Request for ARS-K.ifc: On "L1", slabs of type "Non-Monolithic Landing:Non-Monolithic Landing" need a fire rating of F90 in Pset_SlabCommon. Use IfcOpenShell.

First a look at what the model holds.

```python
import ifcopenshell
import ifcopenshell.util.element

model = ifcopenshell.open("ARS-K.ifc")
print(model.schema)
storey = next(s for s in model.by_type("IfcBuildingStorey") if s.Name == "L1")
slabs = [e for e in ifcopenshell.util.element.get_decomposition(storey) if e.is_a("IfcSlab")]
seen = {}
for e in slabs:
    element_type = ifcopenshell.util.element.get_type(e)
    key = (element_type.Name if element_type != e and element_type else None, ifcopenshell.util.element.get_pset(e, "Pset_SlabCommon", "FireRating"))
    seen[key] = seen.get(key, 0) + 1
for (name, value), count in sorted(seen.items(), key=str):
    print(count, "x", name, "|", value)
```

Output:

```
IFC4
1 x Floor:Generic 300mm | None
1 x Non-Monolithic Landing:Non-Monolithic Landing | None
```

```python
import ifcopenshell
import ifcopenshell.api.pset
import ifcopenshell.util.element

model = ifcopenshell.open("ARS-K.ifc")

storey = next(s for s in model.by_type("IfcBuildingStorey") if s.Name == "L1")
slabs = [e for e in ifcopenshell.util.element.get_decomposition(storey) if e.is_a("IfcSlab")]

count = 0
for e in slabs:
    element_type = ifcopenshell.util.element.get_type(e)
    if element_type in (None, e) or element_type.Name != "Non-Monolithic Landing:Non-Monolithic Landing":
        continue
    # add_pset returns the element's existing set when there is one.
    pset = ifcopenshell.api.pset.add_pset(model, product=e, name="Pset_SlabCommon")
    ifcopenshell.api.pset.edit_pset(model, pset=pset, properties={"FireRating": "F90"})
    count += 1

print(count, "slabs updated")

model.write("ARS-K_edited.ifc")
```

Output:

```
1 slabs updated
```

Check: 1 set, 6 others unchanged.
